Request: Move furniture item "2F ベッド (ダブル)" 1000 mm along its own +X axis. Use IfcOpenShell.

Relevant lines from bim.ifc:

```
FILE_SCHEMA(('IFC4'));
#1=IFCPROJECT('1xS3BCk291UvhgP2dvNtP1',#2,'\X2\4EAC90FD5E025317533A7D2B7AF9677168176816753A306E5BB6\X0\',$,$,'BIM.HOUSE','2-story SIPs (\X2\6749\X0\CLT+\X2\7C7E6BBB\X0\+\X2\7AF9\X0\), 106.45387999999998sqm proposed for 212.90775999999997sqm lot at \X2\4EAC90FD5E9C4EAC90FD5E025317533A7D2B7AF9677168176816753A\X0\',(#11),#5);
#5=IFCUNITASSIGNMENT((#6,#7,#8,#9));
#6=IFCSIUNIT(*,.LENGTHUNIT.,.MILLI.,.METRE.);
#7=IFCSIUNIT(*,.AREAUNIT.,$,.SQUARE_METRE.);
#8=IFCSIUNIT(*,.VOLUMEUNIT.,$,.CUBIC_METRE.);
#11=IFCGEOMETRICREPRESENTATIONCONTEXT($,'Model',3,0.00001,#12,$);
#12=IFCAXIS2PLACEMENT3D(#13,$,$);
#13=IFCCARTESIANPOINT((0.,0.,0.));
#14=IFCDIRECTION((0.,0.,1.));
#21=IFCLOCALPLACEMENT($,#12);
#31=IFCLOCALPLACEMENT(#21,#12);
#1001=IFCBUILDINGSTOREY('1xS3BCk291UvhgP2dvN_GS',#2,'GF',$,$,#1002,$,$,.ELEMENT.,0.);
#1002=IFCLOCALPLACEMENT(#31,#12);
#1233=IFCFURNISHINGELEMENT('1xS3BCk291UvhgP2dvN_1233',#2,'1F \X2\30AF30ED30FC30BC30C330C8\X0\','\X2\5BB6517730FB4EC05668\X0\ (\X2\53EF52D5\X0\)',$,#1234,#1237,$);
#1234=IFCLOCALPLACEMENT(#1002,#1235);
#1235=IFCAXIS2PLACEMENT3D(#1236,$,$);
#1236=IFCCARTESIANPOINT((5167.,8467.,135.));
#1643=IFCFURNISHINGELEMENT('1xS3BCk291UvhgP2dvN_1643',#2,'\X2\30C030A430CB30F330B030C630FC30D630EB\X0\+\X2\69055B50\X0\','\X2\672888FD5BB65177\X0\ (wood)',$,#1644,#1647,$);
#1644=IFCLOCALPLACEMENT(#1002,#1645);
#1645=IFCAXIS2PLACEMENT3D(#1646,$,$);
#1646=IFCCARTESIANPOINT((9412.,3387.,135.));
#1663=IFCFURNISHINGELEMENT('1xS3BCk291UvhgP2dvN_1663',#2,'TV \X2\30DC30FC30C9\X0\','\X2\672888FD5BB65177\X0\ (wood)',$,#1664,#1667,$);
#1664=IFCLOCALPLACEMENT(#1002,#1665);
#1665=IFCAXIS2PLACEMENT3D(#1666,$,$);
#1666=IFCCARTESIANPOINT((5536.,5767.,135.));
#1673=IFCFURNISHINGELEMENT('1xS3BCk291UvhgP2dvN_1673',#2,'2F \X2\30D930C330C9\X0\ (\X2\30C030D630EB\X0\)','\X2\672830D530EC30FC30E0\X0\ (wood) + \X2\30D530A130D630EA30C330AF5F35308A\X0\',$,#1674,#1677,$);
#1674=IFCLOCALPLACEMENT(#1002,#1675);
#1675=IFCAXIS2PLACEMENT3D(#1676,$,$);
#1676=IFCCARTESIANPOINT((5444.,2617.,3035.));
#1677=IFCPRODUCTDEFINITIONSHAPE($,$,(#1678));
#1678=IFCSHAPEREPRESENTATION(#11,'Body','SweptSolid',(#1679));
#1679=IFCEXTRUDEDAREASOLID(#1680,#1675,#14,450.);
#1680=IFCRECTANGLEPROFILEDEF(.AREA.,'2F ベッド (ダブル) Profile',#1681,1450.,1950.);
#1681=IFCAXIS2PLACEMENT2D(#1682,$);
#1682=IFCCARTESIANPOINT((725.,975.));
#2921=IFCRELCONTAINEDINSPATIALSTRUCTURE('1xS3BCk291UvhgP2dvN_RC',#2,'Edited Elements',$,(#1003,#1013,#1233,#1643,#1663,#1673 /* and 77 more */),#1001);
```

```python
import ifcopenshell
import ifcopenshell.api.geometry
import ifcopenshell.util.placement

model = ifcopenshell.open("bim.ifc")

item = model.by_guid("1xS3BCk291UvhgP2dvN_1673")
matrix = ifcopenshell.util.placement.get_local_placement(item.ObjectPlacement)
matrix[:3, 3] += matrix[:3, 0] * 1000.0
ifcopenshell.api.geometry.edit_object_placement(model, product=item, matrix=matrix, is_si=False)

print(ifcopenshell.util.placement.get_local_placement(item.ObjectPlacement).round(3) + 0.0)

model.write("bim_updated.ifc")
```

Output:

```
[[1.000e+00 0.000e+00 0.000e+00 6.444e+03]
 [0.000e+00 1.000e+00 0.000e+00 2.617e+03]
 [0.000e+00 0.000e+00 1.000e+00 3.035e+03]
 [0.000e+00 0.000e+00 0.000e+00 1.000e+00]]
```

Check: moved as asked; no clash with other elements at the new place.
